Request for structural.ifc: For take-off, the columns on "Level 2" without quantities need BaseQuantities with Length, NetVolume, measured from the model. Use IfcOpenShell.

First a look at what the model holds.

```python
import ifcopenshell
import ifcopenshell.util.element
import ifcopenshell.util.unit

model = ifcopenshell.open("structural.ifc")
print(model.schema)
for unit_type in ("LENGTHUNIT", "AREAUNIT", "VOLUMEUNIT"):
    print(unit_type, ifcopenshell.util.unit.calculate_unit_scale(model, unit_type))
storey = next(s for s in model.by_type("IfcBuildingStorey") if s.Name == "Level 2")
columns = [e for e in ifcopenshell.util.element.get_decomposition(storey) if e.is_a("IfcColumn")]
for e in sorted(columns, key=lambda e: e.id()):
    print(e.id(), e.is_a(), e.Name, list(ifcopenshell.util.element.get_psets(e, qtos_only=True)), sep=" | ")
```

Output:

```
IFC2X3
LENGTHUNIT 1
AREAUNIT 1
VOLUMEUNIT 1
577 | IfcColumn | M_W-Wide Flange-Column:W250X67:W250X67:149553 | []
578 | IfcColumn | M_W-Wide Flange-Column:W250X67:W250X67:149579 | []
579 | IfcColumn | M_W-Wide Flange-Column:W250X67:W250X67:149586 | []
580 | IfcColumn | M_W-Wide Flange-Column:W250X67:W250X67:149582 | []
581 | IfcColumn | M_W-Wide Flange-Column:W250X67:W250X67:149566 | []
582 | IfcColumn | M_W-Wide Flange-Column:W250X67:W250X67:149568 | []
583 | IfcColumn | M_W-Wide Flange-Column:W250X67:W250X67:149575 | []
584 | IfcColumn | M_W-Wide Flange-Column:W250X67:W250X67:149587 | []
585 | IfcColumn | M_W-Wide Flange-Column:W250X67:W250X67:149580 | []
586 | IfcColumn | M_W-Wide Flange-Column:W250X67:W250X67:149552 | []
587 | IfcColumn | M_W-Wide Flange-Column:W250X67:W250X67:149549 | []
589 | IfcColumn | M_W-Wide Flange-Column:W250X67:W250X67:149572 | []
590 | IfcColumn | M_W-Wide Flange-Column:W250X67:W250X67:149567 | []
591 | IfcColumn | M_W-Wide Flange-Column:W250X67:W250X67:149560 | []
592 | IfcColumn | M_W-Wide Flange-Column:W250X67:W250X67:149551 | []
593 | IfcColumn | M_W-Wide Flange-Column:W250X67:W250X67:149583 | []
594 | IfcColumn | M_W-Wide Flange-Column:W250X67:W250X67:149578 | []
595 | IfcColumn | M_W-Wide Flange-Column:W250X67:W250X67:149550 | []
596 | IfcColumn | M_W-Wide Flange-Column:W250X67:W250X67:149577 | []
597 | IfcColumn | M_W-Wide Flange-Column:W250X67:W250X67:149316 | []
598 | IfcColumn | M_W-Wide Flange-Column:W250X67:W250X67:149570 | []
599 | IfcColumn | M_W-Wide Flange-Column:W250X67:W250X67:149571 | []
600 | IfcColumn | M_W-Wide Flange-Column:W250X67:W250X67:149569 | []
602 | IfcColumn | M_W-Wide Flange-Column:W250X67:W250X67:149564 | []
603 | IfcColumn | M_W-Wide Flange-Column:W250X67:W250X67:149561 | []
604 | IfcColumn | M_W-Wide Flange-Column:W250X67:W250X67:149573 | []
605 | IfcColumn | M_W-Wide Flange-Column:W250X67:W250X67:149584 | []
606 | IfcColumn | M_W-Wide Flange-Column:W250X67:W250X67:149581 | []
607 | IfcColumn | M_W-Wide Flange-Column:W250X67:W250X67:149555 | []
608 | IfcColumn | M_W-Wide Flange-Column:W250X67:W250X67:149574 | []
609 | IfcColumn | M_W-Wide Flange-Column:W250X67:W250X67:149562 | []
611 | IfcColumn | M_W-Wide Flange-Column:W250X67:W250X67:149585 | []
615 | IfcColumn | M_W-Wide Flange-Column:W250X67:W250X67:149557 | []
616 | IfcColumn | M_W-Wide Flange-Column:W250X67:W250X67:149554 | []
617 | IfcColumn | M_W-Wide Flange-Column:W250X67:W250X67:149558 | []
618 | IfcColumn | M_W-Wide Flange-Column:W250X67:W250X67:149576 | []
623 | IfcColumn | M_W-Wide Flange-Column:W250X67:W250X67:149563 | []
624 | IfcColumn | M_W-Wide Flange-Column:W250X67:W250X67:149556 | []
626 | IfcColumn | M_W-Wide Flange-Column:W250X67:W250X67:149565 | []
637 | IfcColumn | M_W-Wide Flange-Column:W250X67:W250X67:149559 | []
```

```python
import ifcopenshell
import ifcopenshell.api.pset
import ifcopenshell.geom
import ifcopenshell.util.element
import ifcopenshell.util.shape
import ifcopenshell.util.unit

model = ifcopenshell.open("structural.ifc")
unit_scale = ifcopenshell.util.unit.calculate_unit_scale(model)
volume_scale = ifcopenshell.util.unit.calculate_unit_scale(model, "VOLUMEUNIT")
settings = ifcopenshell.geom.settings()

storey = next(s for s in model.by_type("IfcBuildingStorey") if s.Name == "Level 2")
columns = [e for e in ifcopenshell.util.element.get_decomposition(storey) if e.is_a("IfcColumn")]

for e in sorted(columns, key=lambda e: e.id()):
    if ifcopenshell.util.element.get_psets(e, qtos_only=True, should_inherit=False):
        continue
    # Geometry comes back in metres, in the element's own axes.
    shape = ifcopenshell.geom.create_shape(settings, e)
    values = {
        "Length": ifcopenshell.util.shape.get_z(shape.geometry) / unit_scale,
        "NetVolume": ifcopenshell.util.shape.get_volume(shape.geometry) / volume_scale,
    }
    qto = ifcopenshell.api.pset.add_qto(model, product=e, name="BaseQuantities")
    ifcopenshell.api.pset.edit_qto(model, qto=qto, properties=values)
    print(e.id(), {k: round(v, 3) for k, v in values.items()})

model.write("structural_updated.ifc")
```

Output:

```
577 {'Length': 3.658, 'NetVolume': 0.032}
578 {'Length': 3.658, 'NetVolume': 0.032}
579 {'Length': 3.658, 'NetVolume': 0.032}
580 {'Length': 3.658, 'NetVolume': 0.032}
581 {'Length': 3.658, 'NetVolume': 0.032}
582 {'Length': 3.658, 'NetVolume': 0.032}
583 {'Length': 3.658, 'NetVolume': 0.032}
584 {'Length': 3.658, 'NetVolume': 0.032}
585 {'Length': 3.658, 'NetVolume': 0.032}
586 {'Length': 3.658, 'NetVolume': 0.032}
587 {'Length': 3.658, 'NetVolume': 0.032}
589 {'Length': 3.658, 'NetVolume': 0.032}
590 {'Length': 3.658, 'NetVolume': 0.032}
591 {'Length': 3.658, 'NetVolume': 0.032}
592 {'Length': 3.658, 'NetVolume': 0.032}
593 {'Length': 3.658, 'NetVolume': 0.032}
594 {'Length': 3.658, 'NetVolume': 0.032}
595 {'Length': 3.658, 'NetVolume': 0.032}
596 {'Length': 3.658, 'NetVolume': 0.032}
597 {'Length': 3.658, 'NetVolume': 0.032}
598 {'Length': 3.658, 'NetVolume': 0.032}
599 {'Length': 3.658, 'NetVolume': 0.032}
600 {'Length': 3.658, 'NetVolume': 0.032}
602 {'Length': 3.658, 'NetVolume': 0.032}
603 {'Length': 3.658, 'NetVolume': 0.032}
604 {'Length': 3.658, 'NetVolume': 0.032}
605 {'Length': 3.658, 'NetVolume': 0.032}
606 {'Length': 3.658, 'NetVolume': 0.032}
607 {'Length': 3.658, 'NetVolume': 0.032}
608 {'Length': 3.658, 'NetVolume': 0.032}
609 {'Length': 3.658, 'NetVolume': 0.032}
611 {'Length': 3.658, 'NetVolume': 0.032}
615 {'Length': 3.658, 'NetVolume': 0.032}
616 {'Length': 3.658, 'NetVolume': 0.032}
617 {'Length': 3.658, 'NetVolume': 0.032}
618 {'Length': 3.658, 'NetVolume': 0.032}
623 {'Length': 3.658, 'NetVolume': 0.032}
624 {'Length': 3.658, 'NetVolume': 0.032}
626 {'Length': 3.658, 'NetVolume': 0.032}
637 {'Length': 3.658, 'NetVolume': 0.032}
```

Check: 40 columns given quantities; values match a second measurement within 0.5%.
